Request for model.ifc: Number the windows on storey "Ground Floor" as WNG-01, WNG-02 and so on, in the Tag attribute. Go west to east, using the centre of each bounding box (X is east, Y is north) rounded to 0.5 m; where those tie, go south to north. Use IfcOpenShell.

First a look at what the model holds.

```python
import ifcopenshell
import ifcopenshell.util.element
import ifcopenshell.util.placement

model = ifcopenshell.open("model.ifc")
print(model.schema)
storey = next(s for s in model.by_type("IfcBuildingStorey") if s.Name == "Ground Floor")
windows = [e for e in ifcopenshell.util.element.get_decomposition(storey) if e.is_a("IfcWindow")]
for e in sorted(windows, key=lambda e: e.id()):
    origin = ifcopenshell.util.placement.get_local_placement(e.ObjectPlacement)[:3, 3]
    print(e.id(), e.Tag, e.Name, origin.round(2) + 0.0, sep=" | ")
```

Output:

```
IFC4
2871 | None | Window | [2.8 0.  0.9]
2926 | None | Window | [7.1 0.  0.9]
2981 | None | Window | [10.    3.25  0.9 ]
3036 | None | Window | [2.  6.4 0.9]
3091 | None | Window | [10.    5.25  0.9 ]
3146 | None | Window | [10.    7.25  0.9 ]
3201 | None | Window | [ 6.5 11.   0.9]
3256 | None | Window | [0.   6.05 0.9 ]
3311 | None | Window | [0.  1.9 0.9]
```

```python
import ifcopenshell
import ifcopenshell.geom
import ifcopenshell.util.element
import ifcopenshell.util.shape

model = ifcopenshell.open("model.ifc")
settings = ifcopenshell.geom.settings()
settings.set("use-world-coords", True)


def centre(element):
    shape = ifcopenshell.geom.create_shape(settings, element)
    return ifcopenshell.util.shape.get_bbox_centroid(shape.geometry)


storey = next(s for s in model.by_type("IfcBuildingStorey") if s.Name == "Ground Floor")
windows = [e for e in ifcopenshell.util.element.get_decomposition(storey) if e.is_a("IfcWindow")]

# Insertion points can sit at a corner or the storey origin, so sort by the geometry (in metres).
centres = {e: centre(e) for e in windows}
windows.sort(key=lambda e: (round(centres[e][0] / 0.5), centres[e][1]))

for i, e in enumerate(windows, start=1):
    number = f"WNG-{i:02d}"
    e.Tag = number
    print(e.id(), number)

model.write("model_v2.ifc")
```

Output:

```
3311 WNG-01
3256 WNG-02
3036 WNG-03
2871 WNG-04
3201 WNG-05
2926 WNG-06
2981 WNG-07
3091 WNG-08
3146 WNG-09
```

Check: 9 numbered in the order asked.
